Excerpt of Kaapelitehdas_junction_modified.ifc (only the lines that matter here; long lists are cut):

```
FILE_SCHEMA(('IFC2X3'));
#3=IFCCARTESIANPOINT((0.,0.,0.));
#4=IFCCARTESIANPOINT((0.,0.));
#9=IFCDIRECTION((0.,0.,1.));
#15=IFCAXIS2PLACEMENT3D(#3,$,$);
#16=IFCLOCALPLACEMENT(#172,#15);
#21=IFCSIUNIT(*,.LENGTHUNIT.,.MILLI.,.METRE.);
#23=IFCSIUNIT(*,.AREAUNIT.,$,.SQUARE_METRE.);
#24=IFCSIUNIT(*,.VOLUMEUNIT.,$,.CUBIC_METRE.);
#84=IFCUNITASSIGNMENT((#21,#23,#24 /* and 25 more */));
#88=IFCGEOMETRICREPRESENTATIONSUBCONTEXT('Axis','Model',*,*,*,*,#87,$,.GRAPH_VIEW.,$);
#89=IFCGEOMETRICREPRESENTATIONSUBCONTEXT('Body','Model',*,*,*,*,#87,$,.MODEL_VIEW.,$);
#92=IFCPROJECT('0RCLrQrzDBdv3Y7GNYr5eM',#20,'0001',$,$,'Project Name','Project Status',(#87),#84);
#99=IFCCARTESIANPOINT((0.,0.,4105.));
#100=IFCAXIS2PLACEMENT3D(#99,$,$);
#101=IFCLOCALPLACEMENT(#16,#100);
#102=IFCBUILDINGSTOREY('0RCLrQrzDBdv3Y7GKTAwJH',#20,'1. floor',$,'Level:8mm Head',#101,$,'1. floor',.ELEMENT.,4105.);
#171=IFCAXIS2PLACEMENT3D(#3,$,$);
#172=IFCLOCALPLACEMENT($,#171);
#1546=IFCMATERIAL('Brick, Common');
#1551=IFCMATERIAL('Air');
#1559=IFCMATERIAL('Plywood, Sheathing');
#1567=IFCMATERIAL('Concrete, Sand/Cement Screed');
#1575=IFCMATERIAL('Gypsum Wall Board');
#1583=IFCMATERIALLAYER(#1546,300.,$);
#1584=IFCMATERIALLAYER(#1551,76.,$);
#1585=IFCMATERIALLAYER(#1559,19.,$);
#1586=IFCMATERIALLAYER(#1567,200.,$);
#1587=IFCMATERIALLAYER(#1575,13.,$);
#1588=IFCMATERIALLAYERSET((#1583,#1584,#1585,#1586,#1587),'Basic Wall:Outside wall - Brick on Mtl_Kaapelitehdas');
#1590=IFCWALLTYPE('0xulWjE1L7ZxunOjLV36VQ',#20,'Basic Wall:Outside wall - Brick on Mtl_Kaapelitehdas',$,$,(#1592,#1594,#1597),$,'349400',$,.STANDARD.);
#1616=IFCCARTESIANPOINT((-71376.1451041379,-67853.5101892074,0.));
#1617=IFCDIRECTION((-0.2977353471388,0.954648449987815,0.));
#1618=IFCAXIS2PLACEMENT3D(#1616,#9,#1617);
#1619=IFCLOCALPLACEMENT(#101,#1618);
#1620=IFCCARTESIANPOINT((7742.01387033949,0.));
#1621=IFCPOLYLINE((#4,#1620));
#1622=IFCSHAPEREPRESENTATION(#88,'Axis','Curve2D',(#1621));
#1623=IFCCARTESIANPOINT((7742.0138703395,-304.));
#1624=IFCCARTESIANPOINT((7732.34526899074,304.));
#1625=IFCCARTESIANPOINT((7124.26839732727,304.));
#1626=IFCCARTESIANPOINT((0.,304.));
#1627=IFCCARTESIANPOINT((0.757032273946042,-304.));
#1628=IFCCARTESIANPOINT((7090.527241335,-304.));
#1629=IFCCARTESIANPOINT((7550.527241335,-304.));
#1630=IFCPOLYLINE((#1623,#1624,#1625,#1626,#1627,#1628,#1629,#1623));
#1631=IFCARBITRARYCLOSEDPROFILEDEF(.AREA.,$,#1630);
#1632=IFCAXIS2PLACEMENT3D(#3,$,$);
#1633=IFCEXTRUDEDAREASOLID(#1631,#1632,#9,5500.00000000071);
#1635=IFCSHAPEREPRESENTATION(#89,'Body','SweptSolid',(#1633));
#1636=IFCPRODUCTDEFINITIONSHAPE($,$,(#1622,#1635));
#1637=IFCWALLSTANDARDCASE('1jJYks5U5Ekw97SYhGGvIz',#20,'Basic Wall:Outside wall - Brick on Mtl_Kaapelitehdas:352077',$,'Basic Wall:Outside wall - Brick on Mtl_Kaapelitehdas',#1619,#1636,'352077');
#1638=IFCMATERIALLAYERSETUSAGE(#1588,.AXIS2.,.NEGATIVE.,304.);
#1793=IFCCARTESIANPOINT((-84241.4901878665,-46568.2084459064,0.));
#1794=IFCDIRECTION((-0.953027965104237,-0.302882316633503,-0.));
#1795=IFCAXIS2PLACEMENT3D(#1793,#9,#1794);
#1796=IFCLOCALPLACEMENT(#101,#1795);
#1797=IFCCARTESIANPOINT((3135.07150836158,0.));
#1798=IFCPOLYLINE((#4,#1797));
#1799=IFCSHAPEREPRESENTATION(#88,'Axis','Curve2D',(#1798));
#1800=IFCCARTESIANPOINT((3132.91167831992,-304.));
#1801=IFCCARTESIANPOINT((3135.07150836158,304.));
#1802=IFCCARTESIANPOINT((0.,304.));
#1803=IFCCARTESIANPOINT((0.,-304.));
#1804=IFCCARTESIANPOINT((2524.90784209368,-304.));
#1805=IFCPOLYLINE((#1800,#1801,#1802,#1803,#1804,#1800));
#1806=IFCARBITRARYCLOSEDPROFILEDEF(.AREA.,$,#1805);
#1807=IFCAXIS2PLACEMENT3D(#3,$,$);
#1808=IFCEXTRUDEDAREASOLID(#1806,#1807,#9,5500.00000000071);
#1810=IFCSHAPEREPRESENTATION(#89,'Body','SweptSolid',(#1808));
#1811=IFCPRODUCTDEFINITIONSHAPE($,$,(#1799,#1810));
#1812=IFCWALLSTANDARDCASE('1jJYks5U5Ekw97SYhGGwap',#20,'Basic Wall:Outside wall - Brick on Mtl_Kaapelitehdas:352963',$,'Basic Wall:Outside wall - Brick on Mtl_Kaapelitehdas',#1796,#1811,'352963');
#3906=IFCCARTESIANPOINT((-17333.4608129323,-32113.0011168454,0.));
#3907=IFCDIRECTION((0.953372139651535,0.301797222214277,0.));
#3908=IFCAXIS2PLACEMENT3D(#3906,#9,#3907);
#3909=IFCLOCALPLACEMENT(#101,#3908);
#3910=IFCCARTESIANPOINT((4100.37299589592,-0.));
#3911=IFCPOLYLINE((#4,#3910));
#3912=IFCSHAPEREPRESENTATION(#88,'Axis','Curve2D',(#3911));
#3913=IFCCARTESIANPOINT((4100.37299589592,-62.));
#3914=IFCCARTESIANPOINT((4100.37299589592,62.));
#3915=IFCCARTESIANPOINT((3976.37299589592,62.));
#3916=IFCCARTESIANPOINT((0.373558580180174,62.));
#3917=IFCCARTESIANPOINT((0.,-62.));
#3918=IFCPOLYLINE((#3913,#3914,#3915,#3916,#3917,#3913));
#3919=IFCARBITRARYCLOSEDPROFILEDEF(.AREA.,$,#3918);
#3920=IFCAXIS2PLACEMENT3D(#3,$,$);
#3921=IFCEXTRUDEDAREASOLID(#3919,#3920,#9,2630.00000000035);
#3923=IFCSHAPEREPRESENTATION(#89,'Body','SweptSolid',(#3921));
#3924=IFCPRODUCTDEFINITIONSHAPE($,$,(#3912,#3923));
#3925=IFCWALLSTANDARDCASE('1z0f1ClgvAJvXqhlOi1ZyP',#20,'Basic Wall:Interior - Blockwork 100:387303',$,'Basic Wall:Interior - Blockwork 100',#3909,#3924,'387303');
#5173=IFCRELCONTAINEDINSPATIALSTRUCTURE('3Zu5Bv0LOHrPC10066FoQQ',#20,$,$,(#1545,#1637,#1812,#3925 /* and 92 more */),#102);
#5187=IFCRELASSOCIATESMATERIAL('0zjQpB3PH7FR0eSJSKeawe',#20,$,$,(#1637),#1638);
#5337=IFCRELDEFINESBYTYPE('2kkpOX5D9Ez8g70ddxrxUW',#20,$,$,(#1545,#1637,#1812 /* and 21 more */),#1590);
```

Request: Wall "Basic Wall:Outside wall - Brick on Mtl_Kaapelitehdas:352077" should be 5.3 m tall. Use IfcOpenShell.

```python
import ifcopenshell
import ifcopenshell.geom
import ifcopenshell.util.representation
import ifcopenshell.util.shape

model = ifcopenshell.open("Kaapelitehdas_junction_modified.ifc")
settings = ifcopenshell.geom.settings()


def volume(element):
    """Net volume in cubic metres, openings subtracted."""
    shape = ifcopenshell.geom.create_shape(settings, element)
    return ifcopenshell.util.shape.get_volume(shape.geometry)


wall = model.by_guid("1jJYks5U5Ekw97SYhGGvIz")
before = volume(wall)

body = ifcopenshell.util.representation.get_representation(wall, "Model", "Body")
solid = body.Items[0]
old_height = solid.Depth
solid.Depth = 5300.0
after = volume(wall)

print(f"height {old_height:g} -> {solid.Depth:g}, volume {before:.3f} -> {after:.3f} m3")

model.write("Kaapelitehdas_junction_modified_updated.ifc")
```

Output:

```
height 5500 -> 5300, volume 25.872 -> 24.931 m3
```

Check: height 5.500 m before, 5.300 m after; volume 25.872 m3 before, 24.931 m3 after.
